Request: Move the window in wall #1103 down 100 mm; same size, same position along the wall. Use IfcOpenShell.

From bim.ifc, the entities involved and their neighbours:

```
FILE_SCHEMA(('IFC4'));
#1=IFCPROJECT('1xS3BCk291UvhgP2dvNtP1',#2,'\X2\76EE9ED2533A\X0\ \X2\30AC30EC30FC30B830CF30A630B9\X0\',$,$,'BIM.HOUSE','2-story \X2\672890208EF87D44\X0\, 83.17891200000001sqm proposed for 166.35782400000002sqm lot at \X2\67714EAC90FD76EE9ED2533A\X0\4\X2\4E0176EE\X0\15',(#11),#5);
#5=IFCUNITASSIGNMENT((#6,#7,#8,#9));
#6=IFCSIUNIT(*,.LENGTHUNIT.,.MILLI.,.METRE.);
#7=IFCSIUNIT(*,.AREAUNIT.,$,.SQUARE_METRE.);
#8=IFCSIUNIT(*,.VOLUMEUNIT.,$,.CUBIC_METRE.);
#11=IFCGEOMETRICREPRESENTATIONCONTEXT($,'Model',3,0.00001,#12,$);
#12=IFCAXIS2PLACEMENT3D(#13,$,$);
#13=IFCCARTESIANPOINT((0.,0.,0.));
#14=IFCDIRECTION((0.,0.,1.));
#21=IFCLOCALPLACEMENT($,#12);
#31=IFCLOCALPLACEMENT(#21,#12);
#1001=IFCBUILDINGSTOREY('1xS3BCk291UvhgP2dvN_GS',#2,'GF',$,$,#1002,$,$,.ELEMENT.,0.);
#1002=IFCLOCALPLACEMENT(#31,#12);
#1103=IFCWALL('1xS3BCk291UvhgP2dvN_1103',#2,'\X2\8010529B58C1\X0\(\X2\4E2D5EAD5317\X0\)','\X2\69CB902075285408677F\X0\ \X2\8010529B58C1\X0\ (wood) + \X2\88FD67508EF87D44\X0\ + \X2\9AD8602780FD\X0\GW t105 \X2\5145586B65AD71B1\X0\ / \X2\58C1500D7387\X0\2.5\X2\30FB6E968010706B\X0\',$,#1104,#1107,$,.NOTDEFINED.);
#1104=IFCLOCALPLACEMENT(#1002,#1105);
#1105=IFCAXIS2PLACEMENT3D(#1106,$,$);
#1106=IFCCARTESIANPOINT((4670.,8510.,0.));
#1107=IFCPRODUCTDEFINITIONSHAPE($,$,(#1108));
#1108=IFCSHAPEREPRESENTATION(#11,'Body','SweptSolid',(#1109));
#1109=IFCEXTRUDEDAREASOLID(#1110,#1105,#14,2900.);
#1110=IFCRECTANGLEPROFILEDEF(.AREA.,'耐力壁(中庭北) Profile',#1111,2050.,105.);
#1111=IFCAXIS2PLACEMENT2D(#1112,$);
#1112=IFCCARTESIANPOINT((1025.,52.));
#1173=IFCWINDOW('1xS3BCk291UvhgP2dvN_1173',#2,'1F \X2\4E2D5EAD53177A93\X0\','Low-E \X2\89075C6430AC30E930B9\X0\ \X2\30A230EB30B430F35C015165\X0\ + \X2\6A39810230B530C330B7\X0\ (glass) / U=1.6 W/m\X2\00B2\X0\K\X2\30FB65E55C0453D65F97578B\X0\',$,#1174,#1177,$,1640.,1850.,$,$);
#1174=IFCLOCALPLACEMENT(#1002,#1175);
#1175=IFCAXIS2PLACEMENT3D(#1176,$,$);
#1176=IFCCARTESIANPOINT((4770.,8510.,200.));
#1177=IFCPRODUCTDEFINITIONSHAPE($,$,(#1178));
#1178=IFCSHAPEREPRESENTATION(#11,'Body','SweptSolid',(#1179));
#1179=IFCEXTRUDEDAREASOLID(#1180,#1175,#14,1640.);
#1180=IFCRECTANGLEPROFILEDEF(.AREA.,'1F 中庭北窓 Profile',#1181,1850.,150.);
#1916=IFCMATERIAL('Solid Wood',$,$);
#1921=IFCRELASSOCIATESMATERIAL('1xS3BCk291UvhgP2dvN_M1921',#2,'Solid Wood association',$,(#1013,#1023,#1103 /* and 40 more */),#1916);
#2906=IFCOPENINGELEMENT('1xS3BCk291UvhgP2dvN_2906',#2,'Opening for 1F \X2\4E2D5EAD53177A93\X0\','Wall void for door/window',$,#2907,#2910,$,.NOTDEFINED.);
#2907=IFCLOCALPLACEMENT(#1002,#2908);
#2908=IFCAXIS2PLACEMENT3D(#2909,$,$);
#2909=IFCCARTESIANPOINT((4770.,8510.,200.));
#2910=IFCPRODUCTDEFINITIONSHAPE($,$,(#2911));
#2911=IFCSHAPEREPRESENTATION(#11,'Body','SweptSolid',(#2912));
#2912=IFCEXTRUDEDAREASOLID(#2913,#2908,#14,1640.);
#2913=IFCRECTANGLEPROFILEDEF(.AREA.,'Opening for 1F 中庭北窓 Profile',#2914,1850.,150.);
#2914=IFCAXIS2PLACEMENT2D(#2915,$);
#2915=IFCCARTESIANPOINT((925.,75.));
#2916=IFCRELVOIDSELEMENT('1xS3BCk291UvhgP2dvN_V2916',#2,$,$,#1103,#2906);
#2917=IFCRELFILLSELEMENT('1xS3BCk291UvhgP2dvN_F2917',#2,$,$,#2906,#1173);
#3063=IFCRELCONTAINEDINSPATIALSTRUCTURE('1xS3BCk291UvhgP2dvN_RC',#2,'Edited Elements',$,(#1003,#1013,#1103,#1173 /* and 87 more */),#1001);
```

```python
import numpy as np
import ifcopenshell
import ifcopenshell.api.geometry
import ifcopenshell.util.placement
import ifcopenshell.util.unit

model = ifcopenshell.open("bim.ifc")
unit_scale = ifcopenshell.util.unit.calculate_unit_scale(model)

window = model.by_id(1173)
opening = window.FillsVoids[0].RelatingOpeningElement
dz = -0.1 / unit_scale

shift = np.array([0.0, 0.0, dz])
# The window is not placed relative to its opening, so move both.
for product in (opening, window):
    matrix = ifcopenshell.util.placement.get_local_placement(product.ObjectPlacement)
    matrix[:3, 3] += shift
    ifcopenshell.api.geometry.edit_object_placement(model, product=product, matrix=matrix, is_si=False)

print(f"moved by {dz * unit_scale:+.3f} m")

model.write("bim_v2.ifc")
```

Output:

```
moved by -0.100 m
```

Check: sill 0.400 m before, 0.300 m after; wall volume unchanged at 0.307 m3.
